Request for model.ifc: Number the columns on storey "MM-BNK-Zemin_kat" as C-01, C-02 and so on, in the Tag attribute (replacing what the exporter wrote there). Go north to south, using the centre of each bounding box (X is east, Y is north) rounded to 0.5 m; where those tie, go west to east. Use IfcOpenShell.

First a look at what the model holds.

```python
import ifcopenshell
import ifcopenshell.util.element
import ifcopenshell.util.placement

model = ifcopenshell.open("model.ifc")
print(model.schema)
storey = next(s for s in model.by_type("IfcBuildingStorey") if s.Name == "MM-BNK-Zemin_kat")
columns = [e for e in ifcopenshell.util.element.get_decomposition(storey) if e.is_a("IfcColumn")]
for e in sorted(columns, key=lambda e: e.id()):
    origin = ifcopenshell.util.placement.get_local_placement(e.ObjectPlacement)[:3, 3]
    print(e.id(), e.Tag, e.Name, origin.round(2) + 0.0, sep=" | ")
```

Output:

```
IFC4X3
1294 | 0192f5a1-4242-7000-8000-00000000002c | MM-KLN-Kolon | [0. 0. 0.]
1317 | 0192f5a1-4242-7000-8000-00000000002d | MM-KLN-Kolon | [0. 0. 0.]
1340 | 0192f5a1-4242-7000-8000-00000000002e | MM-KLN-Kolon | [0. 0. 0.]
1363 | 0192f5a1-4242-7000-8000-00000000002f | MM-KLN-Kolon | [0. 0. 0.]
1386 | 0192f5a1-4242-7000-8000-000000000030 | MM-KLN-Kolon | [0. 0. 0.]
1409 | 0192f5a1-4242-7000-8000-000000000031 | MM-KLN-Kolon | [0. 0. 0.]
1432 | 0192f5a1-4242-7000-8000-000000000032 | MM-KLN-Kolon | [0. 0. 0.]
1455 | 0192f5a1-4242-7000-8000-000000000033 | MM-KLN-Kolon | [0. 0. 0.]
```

```python
import ifcopenshell
import ifcopenshell.geom
import ifcopenshell.util.element
import ifcopenshell.util.shape

model = ifcopenshell.open("model.ifc")
settings = ifcopenshell.geom.settings()
settings.set("use-world-coords", True)


def centre(element):
    shape = ifcopenshell.geom.create_shape(settings, element)
    return ifcopenshell.util.shape.get_bbox_centroid(shape.geometry)


storey = next(s for s in model.by_type("IfcBuildingStorey") if s.Name == "MM-BNK-Zemin_kat")
columns = [e for e in ifcopenshell.util.element.get_decomposition(storey) if e.is_a("IfcColumn")]

# Insertion points can sit at a corner or the storey origin, so sort by the geometry (in metres).
centres = {e: centre(e) for e in columns}
columns.sort(key=lambda e: (-round(centres[e][1] / 0.5), centres[e][0]))

for i, e in enumerate(columns, start=1):
    number = f"C-{i:02d}"
    e.Tag = number
    print(e.id(), number)

model.write("model_v2.ifc")
```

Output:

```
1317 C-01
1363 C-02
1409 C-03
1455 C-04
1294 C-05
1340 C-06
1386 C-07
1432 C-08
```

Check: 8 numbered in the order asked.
